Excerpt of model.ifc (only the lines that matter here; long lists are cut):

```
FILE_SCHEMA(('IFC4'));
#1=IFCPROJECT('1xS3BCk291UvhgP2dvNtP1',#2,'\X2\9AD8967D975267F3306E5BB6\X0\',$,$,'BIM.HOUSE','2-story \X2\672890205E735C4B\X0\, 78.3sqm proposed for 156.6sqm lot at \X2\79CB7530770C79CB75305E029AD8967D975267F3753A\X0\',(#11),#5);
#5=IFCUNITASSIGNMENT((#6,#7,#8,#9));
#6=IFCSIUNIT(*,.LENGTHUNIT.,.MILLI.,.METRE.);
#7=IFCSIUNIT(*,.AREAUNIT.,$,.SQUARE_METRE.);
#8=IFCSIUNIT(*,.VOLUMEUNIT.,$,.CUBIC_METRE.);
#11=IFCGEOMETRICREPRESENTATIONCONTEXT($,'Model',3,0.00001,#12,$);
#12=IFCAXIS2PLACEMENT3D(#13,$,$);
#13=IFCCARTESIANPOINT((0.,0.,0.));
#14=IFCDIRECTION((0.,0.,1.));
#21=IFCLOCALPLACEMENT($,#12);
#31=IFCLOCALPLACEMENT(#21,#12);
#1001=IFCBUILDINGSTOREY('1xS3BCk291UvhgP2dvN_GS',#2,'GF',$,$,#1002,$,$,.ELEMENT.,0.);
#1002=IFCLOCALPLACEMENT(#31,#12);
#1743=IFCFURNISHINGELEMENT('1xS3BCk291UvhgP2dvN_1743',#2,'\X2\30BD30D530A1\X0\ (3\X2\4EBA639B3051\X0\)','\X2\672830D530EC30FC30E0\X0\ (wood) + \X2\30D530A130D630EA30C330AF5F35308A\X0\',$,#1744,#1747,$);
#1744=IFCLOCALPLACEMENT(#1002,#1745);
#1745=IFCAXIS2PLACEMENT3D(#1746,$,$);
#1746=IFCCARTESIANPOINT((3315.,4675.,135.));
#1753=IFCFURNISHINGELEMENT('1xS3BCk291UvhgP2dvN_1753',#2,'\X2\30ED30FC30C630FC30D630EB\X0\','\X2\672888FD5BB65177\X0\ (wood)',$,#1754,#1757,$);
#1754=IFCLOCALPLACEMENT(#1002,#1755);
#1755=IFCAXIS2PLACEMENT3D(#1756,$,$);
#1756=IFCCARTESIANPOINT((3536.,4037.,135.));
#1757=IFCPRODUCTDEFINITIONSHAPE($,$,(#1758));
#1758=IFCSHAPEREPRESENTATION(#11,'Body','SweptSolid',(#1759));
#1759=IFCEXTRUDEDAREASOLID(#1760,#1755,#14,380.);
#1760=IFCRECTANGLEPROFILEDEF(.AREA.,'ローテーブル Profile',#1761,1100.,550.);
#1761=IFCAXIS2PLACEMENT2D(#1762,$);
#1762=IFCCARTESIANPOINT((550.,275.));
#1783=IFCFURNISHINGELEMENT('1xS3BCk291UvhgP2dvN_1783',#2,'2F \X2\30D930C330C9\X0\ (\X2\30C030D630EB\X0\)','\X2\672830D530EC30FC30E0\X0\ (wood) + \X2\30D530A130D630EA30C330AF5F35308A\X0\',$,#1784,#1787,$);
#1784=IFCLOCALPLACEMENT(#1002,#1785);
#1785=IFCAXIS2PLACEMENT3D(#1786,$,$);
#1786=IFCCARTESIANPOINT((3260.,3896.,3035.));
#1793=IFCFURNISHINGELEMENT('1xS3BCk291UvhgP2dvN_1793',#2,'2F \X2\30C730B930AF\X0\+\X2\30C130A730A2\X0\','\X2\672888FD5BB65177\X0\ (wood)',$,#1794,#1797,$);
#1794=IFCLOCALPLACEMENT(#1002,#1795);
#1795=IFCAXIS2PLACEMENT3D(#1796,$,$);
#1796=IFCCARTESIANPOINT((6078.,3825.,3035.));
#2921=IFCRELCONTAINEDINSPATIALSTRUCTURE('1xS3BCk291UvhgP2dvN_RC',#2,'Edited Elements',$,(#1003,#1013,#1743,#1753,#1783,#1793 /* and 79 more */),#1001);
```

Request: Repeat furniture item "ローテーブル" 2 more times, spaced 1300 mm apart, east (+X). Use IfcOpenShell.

```python
import numpy as np
import ifcopenshell
import ifcopenshell.api.geometry
import ifcopenshell.api.root
import ifcopenshell.util.element
import ifcopenshell.util.placement
import ifcopenshell.util.unit

model = ifcopenshell.open("model.ifc")
unit_scale = ifcopenshell.util.unit.calculate_unit_scale(model)


def reuse_history(source, copy):
    """copy_class also copies each property set's owner history, people and application; keep the originals."""
    for rel in copy.IsDefinedBy:
        if rel.is_a("IfcRelDefinesByProperties") and (history := rel.RelatingPropertyDefinition.OwnerHistory):
            rel.RelatingPropertyDefinition.OwnerHistory = source.OwnerHistory
            ifcopenshell.util.element.remove_deep2(model, history)


source = model.by_id(1753)
base = ifcopenshell.util.placement.get_local_placement(source.ObjectPlacement)
step = np.array([1.0, 0.0, 0.0]) * 1.3 / unit_scale

for i in range(1, 3):
    copy = ifcopenshell.api.root.copy_class(model, product=source)
    copy.Representation = ifcopenshell.util.element.copy_deep(
        model, source.Representation, exclude=["IfcGeometricRepresentationContext", "IfcRepresentationMap"]
    )
    reuse_history(source, copy)
    matrix = base.copy()
    matrix[:3, 3] += i * step
    print("added at", matrix[:3, 3].round(3) + 0.0)
    ifcopenshell.api.geometry.edit_object_placement(model, product=copy, matrix=matrix, is_si=False)

model.write("model-out.ifc")
```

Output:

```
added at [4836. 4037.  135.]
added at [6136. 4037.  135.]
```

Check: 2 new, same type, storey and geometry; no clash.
